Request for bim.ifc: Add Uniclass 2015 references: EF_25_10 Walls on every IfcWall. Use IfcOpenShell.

First a look at what the model holds.

```python
import ifcopenshell

model = ifcopenshell.open("bim.ifc")
print(model.schema)
print("classifications:", [c.Name for c in model.by_type("IfcClassification")])
for ifc_class in ("IfcDoor", "IfcRoof", "IfcStair", "IfcWall", "IfcWindow"):
    print(ifc_class, len(model.by_type(ifc_class)))
```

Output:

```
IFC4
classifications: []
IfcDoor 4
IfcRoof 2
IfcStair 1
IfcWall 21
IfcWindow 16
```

```python
import ifcopenshell
import ifcopenshell.api.classification

model = ifcopenshell.open("bim.ifc")

system = ifcopenshell.api.classification.add_classification(model, classification="Uniclass 2015")

codes = {
    "IfcWall": ("EF_25_10", "Walls"),
}
for ifc_class, (code, name) in codes.items():
    products = model.by_type(ifc_class)
    ifcopenshell.api.classification.add_reference(
        model, products=products, classification=system, identification=code, name=name
    )
    print(code, len(products))

model.write("bim_edited.ifc")
```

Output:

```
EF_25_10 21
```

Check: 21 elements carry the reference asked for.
